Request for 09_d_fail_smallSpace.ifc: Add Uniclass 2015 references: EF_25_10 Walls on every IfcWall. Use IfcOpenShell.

First a look at what the model holds.

```python
import ifcopenshell

model = ifcopenshell.open("09_d_fail_smallSpace.ifc")
print(model.schema)
print("classifications:", [c.Name for c in model.by_type("IfcClassification")])
for ifc_class in ("IfcDoor", "IfcRoof", "IfcStair", "IfcWall", "IfcWindow"):
    print(ifc_class, len(model.by_type(ifc_class)))
```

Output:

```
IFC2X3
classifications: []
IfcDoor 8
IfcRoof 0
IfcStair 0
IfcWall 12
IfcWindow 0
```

```python
import ifcopenshell
import ifcopenshell.api.classification

model = ifcopenshell.open("09_d_fail_smallSpace.ifc")

# IFC2X3 requires Source and Edition and has no link from the project to the system.
system = model.create_entity("IfcClassification", Source="NBS", Edition="2015", Name="Uniclass 2015")

codes = {
    "IfcWall": ("EF_25_10", "Walls"),
}
for ifc_class, (code, name) in codes.items():
    products = model.by_type(ifc_class)
    ifcopenshell.api.classification.add_reference(
        model, products=products, classification=system, identification=code, name=name
    )
    print(code, len(products))

model.write("09_d_fail_smallSpace-out.ifc")
```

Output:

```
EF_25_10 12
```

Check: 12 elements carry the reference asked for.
